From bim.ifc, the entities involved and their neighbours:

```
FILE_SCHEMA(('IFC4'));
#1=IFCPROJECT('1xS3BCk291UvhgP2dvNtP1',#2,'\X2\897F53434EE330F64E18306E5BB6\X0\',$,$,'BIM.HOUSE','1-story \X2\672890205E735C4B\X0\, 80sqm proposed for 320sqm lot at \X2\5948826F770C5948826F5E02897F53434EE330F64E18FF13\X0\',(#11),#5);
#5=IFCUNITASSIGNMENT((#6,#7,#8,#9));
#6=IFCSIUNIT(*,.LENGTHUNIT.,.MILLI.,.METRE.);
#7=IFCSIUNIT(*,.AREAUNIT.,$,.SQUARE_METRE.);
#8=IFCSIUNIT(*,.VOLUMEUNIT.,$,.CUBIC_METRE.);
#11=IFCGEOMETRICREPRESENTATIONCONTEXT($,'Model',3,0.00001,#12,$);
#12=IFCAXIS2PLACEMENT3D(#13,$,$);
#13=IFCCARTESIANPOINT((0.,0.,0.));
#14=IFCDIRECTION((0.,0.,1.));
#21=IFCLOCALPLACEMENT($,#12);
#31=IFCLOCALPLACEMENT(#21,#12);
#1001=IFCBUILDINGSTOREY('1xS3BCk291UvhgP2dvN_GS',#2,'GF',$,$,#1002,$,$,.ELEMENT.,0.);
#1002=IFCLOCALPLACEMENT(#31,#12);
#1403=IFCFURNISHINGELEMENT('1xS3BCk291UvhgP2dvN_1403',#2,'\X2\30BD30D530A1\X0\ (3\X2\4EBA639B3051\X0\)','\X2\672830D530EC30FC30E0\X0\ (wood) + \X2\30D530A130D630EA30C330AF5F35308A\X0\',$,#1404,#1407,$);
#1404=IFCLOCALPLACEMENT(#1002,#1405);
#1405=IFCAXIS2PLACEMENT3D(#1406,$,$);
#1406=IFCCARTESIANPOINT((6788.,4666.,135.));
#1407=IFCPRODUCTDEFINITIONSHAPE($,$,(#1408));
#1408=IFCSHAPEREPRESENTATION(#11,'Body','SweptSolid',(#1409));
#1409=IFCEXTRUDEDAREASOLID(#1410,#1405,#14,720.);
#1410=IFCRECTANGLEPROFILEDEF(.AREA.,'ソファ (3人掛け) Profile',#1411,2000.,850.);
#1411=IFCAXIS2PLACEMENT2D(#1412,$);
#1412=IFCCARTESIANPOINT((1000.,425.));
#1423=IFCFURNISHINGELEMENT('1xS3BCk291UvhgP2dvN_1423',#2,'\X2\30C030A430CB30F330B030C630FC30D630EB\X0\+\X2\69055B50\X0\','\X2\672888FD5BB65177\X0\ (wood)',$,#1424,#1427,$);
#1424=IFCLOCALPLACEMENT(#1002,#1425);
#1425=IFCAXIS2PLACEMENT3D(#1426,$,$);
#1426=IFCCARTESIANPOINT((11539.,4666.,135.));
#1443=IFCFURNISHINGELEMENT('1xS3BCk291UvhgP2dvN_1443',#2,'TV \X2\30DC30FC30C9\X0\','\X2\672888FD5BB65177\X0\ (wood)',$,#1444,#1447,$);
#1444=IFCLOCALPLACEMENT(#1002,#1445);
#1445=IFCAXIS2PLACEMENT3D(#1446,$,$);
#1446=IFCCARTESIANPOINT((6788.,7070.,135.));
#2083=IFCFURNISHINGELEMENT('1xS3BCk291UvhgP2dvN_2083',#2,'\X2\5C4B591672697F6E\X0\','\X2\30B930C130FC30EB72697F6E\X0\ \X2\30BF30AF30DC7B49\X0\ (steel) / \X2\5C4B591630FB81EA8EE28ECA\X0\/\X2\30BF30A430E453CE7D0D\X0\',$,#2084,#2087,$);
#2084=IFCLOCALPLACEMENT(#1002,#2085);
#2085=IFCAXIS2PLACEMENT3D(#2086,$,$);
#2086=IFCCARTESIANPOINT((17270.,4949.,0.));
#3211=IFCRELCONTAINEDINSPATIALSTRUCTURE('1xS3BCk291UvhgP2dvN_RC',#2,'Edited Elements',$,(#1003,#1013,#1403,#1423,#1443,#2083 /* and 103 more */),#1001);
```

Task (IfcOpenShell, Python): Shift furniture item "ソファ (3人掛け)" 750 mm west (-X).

```python
import ifcopenshell
import ifcopenshell.api.geometry
import ifcopenshell.util.placement
import ifcopenshell.util.unit

model = ifcopenshell.open("bim.ifc")
unit_scale = ifcopenshell.util.unit.calculate_unit_scale(model)

item = model.by_guid("1xS3BCk291UvhgP2dvN_1403")
matrix = ifcopenshell.util.placement.get_local_placement(item.ObjectPlacement)
matrix[0, 3] -= 0.75 / unit_scale
ifcopenshell.api.geometry.edit_object_placement(model, product=item, matrix=matrix, is_si=False)

print(ifcopenshell.util.placement.get_local_placement(item.ObjectPlacement).round(3) + 0.0)

model.write("bim-out.ifc")
```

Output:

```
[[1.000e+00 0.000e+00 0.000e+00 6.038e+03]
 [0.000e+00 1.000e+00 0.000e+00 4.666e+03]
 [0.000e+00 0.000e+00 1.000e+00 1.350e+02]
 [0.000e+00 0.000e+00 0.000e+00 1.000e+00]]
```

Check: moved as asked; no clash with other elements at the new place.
